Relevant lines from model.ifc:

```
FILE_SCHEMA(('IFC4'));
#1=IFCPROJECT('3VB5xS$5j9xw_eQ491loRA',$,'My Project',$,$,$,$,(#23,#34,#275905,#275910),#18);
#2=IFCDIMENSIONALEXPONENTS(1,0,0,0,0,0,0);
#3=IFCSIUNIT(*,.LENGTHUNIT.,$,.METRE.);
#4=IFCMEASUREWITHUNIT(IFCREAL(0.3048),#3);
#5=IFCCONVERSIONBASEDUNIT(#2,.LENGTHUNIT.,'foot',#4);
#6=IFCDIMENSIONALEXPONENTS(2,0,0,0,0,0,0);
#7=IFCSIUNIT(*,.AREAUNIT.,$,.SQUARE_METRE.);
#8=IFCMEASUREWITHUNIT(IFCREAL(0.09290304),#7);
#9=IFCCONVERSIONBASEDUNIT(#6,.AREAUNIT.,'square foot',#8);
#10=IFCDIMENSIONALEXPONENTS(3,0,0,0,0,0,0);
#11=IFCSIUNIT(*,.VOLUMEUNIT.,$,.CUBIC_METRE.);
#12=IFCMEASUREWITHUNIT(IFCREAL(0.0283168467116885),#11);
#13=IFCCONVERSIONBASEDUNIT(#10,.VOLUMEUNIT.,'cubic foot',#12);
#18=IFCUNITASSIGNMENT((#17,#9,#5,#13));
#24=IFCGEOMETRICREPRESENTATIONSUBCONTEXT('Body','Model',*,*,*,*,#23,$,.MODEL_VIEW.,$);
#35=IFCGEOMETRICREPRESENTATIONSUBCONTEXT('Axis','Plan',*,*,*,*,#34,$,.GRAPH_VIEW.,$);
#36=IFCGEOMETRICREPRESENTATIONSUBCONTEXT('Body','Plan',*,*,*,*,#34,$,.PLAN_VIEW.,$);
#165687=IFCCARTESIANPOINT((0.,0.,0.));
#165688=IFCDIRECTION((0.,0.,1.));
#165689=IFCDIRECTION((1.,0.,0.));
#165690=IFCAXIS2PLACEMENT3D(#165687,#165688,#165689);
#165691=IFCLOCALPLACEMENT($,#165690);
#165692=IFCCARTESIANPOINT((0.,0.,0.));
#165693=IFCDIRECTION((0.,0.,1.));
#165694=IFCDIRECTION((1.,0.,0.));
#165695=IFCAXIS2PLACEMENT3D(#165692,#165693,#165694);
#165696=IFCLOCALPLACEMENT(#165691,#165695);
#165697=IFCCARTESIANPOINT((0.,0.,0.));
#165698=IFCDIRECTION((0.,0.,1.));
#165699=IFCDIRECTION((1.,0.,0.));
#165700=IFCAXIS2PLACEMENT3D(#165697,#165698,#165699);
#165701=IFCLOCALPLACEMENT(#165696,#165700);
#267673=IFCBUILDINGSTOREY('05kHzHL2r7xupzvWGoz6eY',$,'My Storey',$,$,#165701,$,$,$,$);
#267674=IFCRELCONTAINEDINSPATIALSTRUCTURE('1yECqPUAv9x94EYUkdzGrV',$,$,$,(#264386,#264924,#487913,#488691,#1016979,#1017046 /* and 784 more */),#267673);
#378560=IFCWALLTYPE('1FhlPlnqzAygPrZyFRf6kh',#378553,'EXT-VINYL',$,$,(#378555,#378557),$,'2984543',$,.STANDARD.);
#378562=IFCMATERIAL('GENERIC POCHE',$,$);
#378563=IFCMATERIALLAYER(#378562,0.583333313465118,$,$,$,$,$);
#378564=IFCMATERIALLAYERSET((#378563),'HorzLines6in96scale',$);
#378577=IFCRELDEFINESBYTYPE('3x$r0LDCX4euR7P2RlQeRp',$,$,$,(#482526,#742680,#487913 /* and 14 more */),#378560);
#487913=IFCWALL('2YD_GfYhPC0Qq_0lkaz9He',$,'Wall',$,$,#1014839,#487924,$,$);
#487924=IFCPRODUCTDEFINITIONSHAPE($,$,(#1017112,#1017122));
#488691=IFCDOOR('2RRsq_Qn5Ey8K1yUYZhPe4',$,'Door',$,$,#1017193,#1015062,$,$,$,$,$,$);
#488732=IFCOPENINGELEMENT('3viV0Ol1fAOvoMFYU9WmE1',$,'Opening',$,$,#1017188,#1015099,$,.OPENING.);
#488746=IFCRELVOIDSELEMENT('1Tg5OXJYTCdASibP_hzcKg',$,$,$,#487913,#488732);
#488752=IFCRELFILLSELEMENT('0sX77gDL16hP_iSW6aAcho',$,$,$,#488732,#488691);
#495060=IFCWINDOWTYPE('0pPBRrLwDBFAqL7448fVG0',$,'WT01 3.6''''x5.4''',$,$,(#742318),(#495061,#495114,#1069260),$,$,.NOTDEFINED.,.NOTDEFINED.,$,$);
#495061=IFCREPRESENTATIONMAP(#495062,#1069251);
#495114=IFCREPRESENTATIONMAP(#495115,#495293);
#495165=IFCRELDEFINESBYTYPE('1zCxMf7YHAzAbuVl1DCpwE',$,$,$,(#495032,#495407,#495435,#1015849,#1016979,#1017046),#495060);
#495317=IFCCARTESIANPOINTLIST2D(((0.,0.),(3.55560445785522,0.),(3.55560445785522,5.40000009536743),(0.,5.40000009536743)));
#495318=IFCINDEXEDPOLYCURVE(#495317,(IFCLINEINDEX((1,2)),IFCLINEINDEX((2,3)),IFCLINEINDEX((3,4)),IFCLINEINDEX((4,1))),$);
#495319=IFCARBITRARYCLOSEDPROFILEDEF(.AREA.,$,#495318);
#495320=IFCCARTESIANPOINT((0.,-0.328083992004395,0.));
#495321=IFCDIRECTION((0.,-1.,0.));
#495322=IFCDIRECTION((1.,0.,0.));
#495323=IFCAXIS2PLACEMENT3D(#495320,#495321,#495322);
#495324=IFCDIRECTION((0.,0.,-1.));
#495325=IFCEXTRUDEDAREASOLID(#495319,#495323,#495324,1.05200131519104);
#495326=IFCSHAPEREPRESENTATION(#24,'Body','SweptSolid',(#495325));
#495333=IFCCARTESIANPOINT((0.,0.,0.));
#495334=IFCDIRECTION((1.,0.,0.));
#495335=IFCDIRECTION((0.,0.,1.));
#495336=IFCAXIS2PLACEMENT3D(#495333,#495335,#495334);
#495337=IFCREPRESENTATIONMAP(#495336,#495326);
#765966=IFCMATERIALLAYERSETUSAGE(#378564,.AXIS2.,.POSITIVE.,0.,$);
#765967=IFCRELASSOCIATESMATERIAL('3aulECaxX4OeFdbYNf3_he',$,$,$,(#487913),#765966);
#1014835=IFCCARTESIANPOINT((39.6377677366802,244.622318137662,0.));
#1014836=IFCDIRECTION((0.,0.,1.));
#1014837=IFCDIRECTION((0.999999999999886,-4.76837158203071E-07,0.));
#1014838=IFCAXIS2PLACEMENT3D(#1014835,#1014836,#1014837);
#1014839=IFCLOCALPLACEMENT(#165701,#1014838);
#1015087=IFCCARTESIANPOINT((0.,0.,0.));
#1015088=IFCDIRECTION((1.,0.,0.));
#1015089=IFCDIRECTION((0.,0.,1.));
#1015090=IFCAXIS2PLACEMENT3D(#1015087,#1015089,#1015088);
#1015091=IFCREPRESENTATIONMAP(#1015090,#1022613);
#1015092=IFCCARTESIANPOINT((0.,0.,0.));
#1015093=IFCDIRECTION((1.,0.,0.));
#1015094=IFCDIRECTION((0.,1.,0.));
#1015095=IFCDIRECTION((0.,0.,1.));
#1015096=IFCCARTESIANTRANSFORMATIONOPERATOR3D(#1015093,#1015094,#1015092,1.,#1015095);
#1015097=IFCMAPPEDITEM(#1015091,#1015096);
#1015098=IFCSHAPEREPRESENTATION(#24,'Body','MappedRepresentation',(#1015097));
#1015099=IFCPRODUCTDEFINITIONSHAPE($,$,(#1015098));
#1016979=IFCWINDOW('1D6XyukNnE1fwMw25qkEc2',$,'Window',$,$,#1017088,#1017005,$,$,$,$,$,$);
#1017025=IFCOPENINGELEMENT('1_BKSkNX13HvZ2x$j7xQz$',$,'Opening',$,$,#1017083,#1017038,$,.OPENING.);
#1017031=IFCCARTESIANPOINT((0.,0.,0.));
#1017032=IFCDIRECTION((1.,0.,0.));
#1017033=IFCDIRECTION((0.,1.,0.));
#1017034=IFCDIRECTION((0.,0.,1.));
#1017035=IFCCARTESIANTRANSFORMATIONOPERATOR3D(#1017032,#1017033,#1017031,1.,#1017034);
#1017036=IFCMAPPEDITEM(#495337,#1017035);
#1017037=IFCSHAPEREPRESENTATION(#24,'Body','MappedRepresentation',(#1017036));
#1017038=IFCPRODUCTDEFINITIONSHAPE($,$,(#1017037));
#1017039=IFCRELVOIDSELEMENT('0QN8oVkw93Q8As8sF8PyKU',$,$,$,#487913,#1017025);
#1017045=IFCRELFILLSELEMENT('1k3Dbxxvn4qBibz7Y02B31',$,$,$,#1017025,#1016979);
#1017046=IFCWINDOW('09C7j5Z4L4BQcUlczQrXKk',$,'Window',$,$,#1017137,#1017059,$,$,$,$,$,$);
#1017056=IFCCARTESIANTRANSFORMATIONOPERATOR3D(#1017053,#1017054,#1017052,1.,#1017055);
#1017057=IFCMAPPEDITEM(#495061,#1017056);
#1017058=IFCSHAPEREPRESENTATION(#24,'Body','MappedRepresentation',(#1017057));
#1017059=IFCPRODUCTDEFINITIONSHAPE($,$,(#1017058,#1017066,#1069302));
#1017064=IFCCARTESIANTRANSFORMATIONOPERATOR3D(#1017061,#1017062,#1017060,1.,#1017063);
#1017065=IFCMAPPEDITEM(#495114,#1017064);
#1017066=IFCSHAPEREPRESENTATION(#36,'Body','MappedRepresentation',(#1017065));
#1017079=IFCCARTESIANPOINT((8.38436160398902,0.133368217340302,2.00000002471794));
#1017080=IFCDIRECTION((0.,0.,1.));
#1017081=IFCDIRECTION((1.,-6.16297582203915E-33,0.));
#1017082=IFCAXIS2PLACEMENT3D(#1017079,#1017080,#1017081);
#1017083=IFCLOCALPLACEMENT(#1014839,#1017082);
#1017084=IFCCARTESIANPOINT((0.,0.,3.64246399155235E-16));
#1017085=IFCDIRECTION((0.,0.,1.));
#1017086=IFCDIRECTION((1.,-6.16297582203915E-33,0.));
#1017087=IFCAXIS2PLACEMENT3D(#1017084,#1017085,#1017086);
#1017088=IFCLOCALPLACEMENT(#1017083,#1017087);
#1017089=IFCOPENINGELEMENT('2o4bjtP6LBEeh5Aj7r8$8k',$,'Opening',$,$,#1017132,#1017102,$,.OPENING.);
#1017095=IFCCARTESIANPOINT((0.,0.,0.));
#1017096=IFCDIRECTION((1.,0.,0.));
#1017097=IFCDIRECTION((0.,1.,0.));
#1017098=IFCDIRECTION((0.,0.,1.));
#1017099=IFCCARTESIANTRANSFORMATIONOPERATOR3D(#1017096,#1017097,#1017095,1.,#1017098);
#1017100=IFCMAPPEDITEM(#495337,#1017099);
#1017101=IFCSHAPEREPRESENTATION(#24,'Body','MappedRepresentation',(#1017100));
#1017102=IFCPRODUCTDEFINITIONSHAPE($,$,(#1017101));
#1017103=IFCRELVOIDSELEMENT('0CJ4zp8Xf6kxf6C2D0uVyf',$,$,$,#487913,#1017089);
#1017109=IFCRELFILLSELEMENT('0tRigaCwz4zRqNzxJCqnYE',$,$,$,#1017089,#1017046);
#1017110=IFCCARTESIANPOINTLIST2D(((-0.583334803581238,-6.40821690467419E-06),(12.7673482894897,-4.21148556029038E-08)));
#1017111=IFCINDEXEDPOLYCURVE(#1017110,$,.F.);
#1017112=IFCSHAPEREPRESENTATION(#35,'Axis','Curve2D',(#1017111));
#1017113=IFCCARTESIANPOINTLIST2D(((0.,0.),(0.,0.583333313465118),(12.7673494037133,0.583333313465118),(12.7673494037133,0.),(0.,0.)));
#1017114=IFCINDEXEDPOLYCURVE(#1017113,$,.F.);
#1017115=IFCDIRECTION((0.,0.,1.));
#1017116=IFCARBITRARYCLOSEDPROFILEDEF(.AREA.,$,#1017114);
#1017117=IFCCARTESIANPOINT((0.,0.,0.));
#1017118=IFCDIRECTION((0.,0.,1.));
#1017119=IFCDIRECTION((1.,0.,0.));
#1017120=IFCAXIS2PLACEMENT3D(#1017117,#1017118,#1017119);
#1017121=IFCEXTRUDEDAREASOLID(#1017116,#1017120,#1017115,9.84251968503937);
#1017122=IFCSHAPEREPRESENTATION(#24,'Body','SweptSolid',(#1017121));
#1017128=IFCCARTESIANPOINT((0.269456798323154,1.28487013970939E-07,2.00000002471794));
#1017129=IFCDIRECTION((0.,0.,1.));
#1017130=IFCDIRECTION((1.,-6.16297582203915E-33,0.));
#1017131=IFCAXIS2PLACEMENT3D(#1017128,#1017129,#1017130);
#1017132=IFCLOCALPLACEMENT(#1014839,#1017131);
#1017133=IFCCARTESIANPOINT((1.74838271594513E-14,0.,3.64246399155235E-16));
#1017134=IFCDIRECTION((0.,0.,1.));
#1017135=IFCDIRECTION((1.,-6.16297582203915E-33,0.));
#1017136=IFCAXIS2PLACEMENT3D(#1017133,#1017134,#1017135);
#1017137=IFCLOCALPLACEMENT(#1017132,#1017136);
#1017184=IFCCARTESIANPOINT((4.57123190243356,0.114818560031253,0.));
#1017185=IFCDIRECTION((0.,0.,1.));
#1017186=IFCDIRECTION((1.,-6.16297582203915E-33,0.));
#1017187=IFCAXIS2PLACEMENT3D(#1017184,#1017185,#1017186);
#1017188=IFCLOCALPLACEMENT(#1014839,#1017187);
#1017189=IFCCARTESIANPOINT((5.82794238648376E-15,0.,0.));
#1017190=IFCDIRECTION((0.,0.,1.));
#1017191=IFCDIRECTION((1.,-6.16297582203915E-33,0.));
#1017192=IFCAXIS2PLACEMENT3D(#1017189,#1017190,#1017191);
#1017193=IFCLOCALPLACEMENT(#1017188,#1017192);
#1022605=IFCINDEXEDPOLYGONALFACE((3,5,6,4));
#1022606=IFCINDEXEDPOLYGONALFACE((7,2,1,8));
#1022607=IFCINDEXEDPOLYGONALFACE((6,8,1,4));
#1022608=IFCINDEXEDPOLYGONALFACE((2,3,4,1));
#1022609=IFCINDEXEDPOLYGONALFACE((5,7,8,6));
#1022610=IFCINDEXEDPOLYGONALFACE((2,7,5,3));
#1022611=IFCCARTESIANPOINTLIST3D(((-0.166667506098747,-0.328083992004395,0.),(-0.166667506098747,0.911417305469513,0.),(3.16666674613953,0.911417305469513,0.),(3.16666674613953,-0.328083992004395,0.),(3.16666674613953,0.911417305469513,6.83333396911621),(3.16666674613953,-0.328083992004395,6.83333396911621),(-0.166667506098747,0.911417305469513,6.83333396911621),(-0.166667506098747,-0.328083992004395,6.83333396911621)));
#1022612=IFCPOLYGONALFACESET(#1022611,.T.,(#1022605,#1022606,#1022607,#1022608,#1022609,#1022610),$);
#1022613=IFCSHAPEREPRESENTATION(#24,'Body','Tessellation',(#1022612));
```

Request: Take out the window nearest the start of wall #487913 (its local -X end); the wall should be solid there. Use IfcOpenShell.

```python
import ifcopenshell
import ifcopenshell.api.feature
import ifcopenshell.api.root
import ifcopenshell.geom
import ifcopenshell.util.shape

model = ifcopenshell.open("model.ifc")
settings = ifcopenshell.geom.settings()


def volume(element):
    """Net volume in cubic metres, openings subtracted."""
    shape = ifcopenshell.geom.create_shape(settings, element)
    return ifcopenshell.util.shape.get_volume(shape.geometry)


window = model.by_id(1017046)
opening = window.FillsVoids[0].RelatingOpeningElement
wall = opening.VoidsElements[0].RelatingBuildingElement
before = volume(wall)

ifcopenshell.api.root.remove_product(model, product=window)
ifcopenshell.api.feature.remove_feature(model, feature=opening)

after = volume(wall)

print(f"wall volume {before:.3f} -> {after:.3f} m3")

model.write("model_v2.ifc")
```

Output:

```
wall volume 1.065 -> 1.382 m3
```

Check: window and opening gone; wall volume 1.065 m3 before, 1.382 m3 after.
